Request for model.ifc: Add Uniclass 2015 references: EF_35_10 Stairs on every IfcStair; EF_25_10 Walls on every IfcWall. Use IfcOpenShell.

First a look at what the model holds.

```python
import ifcopenshell

model = ifcopenshell.open("model.ifc")
print(model.schema)
print("classifications:", [c.Name for c in model.by_type("IfcClassification")])
for ifc_class in ("IfcDoor", "IfcRoof", "IfcStair", "IfcWall", "IfcWindow"):
    print(ifc_class, len(model.by_type(ifc_class)))
```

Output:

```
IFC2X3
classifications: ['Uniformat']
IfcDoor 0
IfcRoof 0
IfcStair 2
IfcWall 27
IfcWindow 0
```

```python
import ifcopenshell
import ifcopenshell.api.classification

model = ifcopenshell.open("model.ifc")

# IFC2X3 requires Source and Edition and has no link from the project to the system.
system = model.create_entity("IfcClassification", Source="NBS", Edition="2015", Name="Uniclass 2015")

codes = {
    "IfcStair": ("EF_35_10", "Stairs"),
    "IfcWall": ("EF_25_10", "Walls"),
}
for ifc_class, (code, name) in codes.items():
    products = model.by_type(ifc_class)
    ifcopenshell.api.classification.add_reference(
        model, products=products, classification=system, identification=code, name=name
    )
    print(code, len(products))

model.write("model_updated.ifc")
```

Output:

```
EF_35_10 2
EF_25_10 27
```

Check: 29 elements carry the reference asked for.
